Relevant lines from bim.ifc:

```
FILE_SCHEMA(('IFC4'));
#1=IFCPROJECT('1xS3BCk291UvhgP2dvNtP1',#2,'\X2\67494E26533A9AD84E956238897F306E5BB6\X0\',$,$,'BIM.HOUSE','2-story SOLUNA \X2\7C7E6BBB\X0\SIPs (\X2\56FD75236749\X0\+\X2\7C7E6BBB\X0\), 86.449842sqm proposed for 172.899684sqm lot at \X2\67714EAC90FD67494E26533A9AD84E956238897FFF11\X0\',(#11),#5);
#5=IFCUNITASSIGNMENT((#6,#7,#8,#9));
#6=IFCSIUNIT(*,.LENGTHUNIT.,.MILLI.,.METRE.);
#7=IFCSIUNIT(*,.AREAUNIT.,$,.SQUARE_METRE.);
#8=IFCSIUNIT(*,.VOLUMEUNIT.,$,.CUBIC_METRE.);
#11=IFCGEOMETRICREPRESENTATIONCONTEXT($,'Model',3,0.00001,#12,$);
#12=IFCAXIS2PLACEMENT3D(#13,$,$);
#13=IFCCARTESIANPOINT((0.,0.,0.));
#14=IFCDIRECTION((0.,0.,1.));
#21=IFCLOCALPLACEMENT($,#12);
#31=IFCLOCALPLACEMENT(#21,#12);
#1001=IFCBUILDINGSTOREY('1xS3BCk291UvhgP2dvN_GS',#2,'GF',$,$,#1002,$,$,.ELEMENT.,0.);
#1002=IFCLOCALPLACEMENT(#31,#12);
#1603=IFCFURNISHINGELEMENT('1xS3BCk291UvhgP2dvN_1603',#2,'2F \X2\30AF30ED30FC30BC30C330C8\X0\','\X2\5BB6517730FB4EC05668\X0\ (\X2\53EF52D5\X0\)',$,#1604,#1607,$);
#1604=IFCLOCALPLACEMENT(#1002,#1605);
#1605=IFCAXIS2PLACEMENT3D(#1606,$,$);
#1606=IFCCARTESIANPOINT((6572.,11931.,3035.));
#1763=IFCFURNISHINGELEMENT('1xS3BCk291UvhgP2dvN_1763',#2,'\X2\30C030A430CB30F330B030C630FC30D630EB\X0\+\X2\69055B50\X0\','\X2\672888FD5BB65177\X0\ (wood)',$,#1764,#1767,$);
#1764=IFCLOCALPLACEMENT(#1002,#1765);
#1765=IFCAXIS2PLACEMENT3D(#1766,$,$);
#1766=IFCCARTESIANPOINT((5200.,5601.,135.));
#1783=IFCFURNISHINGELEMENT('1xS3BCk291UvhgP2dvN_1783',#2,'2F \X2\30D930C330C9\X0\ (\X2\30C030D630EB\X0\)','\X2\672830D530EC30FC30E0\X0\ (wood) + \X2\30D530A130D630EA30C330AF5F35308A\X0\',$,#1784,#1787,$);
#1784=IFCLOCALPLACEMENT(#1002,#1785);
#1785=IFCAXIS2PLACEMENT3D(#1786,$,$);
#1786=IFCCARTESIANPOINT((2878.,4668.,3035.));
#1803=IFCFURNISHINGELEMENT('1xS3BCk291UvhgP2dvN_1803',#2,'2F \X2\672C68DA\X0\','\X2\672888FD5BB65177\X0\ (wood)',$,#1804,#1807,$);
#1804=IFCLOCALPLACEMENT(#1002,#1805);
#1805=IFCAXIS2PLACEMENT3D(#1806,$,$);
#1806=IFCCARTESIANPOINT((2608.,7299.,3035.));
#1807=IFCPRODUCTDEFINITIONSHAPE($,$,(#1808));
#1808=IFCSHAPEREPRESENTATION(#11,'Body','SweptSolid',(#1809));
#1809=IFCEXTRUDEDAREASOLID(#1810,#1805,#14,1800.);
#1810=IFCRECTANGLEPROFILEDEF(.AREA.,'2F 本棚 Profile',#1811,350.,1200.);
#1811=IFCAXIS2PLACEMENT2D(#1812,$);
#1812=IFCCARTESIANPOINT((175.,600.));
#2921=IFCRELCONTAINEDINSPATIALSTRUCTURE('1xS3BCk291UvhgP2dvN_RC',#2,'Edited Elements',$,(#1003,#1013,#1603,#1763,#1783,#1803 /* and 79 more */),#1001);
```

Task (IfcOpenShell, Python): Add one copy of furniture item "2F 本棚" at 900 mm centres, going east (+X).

```python
import numpy as np
import ifcopenshell
import ifcopenshell.api.geometry
import ifcopenshell.api.root
import ifcopenshell.util.element
import ifcopenshell.util.placement
import ifcopenshell.util.unit

model = ifcopenshell.open("bim.ifc")
unit_scale = ifcopenshell.util.unit.calculate_unit_scale(model)


def reuse_history(source, copy):
    """copy_class also copies each property set's owner history, people and application; keep the originals."""
    for rel in copy.IsDefinedBy:
        if rel.is_a("IfcRelDefinesByProperties") and (history := rel.RelatingPropertyDefinition.OwnerHistory):
            rel.RelatingPropertyDefinition.OwnerHistory = source.OwnerHistory
            ifcopenshell.util.element.remove_deep2(model, history)


source = model.by_id(1803)
base = ifcopenshell.util.placement.get_local_placement(source.ObjectPlacement)
step = np.array([1.0, 0.0, 0.0]) * 0.9 / unit_scale

for i in range(1, 2):
    copy = ifcopenshell.api.root.copy_class(model, product=source)
    copy.Representation = ifcopenshell.util.element.copy_deep(
        model, source.Representation, exclude=["IfcGeometricRepresentationContext", "IfcRepresentationMap"]
    )
    reuse_history(source, copy)
    matrix = base.copy()
    matrix[:3, 3] += i * step
    print("added at", matrix[:3, 3].round(3) + 0.0)
    ifcopenshell.api.geometry.edit_object_placement(model, product=copy, matrix=matrix, is_si=False)

model.write("bim_v2.ifc")
```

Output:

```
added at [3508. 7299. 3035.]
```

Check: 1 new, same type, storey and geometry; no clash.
